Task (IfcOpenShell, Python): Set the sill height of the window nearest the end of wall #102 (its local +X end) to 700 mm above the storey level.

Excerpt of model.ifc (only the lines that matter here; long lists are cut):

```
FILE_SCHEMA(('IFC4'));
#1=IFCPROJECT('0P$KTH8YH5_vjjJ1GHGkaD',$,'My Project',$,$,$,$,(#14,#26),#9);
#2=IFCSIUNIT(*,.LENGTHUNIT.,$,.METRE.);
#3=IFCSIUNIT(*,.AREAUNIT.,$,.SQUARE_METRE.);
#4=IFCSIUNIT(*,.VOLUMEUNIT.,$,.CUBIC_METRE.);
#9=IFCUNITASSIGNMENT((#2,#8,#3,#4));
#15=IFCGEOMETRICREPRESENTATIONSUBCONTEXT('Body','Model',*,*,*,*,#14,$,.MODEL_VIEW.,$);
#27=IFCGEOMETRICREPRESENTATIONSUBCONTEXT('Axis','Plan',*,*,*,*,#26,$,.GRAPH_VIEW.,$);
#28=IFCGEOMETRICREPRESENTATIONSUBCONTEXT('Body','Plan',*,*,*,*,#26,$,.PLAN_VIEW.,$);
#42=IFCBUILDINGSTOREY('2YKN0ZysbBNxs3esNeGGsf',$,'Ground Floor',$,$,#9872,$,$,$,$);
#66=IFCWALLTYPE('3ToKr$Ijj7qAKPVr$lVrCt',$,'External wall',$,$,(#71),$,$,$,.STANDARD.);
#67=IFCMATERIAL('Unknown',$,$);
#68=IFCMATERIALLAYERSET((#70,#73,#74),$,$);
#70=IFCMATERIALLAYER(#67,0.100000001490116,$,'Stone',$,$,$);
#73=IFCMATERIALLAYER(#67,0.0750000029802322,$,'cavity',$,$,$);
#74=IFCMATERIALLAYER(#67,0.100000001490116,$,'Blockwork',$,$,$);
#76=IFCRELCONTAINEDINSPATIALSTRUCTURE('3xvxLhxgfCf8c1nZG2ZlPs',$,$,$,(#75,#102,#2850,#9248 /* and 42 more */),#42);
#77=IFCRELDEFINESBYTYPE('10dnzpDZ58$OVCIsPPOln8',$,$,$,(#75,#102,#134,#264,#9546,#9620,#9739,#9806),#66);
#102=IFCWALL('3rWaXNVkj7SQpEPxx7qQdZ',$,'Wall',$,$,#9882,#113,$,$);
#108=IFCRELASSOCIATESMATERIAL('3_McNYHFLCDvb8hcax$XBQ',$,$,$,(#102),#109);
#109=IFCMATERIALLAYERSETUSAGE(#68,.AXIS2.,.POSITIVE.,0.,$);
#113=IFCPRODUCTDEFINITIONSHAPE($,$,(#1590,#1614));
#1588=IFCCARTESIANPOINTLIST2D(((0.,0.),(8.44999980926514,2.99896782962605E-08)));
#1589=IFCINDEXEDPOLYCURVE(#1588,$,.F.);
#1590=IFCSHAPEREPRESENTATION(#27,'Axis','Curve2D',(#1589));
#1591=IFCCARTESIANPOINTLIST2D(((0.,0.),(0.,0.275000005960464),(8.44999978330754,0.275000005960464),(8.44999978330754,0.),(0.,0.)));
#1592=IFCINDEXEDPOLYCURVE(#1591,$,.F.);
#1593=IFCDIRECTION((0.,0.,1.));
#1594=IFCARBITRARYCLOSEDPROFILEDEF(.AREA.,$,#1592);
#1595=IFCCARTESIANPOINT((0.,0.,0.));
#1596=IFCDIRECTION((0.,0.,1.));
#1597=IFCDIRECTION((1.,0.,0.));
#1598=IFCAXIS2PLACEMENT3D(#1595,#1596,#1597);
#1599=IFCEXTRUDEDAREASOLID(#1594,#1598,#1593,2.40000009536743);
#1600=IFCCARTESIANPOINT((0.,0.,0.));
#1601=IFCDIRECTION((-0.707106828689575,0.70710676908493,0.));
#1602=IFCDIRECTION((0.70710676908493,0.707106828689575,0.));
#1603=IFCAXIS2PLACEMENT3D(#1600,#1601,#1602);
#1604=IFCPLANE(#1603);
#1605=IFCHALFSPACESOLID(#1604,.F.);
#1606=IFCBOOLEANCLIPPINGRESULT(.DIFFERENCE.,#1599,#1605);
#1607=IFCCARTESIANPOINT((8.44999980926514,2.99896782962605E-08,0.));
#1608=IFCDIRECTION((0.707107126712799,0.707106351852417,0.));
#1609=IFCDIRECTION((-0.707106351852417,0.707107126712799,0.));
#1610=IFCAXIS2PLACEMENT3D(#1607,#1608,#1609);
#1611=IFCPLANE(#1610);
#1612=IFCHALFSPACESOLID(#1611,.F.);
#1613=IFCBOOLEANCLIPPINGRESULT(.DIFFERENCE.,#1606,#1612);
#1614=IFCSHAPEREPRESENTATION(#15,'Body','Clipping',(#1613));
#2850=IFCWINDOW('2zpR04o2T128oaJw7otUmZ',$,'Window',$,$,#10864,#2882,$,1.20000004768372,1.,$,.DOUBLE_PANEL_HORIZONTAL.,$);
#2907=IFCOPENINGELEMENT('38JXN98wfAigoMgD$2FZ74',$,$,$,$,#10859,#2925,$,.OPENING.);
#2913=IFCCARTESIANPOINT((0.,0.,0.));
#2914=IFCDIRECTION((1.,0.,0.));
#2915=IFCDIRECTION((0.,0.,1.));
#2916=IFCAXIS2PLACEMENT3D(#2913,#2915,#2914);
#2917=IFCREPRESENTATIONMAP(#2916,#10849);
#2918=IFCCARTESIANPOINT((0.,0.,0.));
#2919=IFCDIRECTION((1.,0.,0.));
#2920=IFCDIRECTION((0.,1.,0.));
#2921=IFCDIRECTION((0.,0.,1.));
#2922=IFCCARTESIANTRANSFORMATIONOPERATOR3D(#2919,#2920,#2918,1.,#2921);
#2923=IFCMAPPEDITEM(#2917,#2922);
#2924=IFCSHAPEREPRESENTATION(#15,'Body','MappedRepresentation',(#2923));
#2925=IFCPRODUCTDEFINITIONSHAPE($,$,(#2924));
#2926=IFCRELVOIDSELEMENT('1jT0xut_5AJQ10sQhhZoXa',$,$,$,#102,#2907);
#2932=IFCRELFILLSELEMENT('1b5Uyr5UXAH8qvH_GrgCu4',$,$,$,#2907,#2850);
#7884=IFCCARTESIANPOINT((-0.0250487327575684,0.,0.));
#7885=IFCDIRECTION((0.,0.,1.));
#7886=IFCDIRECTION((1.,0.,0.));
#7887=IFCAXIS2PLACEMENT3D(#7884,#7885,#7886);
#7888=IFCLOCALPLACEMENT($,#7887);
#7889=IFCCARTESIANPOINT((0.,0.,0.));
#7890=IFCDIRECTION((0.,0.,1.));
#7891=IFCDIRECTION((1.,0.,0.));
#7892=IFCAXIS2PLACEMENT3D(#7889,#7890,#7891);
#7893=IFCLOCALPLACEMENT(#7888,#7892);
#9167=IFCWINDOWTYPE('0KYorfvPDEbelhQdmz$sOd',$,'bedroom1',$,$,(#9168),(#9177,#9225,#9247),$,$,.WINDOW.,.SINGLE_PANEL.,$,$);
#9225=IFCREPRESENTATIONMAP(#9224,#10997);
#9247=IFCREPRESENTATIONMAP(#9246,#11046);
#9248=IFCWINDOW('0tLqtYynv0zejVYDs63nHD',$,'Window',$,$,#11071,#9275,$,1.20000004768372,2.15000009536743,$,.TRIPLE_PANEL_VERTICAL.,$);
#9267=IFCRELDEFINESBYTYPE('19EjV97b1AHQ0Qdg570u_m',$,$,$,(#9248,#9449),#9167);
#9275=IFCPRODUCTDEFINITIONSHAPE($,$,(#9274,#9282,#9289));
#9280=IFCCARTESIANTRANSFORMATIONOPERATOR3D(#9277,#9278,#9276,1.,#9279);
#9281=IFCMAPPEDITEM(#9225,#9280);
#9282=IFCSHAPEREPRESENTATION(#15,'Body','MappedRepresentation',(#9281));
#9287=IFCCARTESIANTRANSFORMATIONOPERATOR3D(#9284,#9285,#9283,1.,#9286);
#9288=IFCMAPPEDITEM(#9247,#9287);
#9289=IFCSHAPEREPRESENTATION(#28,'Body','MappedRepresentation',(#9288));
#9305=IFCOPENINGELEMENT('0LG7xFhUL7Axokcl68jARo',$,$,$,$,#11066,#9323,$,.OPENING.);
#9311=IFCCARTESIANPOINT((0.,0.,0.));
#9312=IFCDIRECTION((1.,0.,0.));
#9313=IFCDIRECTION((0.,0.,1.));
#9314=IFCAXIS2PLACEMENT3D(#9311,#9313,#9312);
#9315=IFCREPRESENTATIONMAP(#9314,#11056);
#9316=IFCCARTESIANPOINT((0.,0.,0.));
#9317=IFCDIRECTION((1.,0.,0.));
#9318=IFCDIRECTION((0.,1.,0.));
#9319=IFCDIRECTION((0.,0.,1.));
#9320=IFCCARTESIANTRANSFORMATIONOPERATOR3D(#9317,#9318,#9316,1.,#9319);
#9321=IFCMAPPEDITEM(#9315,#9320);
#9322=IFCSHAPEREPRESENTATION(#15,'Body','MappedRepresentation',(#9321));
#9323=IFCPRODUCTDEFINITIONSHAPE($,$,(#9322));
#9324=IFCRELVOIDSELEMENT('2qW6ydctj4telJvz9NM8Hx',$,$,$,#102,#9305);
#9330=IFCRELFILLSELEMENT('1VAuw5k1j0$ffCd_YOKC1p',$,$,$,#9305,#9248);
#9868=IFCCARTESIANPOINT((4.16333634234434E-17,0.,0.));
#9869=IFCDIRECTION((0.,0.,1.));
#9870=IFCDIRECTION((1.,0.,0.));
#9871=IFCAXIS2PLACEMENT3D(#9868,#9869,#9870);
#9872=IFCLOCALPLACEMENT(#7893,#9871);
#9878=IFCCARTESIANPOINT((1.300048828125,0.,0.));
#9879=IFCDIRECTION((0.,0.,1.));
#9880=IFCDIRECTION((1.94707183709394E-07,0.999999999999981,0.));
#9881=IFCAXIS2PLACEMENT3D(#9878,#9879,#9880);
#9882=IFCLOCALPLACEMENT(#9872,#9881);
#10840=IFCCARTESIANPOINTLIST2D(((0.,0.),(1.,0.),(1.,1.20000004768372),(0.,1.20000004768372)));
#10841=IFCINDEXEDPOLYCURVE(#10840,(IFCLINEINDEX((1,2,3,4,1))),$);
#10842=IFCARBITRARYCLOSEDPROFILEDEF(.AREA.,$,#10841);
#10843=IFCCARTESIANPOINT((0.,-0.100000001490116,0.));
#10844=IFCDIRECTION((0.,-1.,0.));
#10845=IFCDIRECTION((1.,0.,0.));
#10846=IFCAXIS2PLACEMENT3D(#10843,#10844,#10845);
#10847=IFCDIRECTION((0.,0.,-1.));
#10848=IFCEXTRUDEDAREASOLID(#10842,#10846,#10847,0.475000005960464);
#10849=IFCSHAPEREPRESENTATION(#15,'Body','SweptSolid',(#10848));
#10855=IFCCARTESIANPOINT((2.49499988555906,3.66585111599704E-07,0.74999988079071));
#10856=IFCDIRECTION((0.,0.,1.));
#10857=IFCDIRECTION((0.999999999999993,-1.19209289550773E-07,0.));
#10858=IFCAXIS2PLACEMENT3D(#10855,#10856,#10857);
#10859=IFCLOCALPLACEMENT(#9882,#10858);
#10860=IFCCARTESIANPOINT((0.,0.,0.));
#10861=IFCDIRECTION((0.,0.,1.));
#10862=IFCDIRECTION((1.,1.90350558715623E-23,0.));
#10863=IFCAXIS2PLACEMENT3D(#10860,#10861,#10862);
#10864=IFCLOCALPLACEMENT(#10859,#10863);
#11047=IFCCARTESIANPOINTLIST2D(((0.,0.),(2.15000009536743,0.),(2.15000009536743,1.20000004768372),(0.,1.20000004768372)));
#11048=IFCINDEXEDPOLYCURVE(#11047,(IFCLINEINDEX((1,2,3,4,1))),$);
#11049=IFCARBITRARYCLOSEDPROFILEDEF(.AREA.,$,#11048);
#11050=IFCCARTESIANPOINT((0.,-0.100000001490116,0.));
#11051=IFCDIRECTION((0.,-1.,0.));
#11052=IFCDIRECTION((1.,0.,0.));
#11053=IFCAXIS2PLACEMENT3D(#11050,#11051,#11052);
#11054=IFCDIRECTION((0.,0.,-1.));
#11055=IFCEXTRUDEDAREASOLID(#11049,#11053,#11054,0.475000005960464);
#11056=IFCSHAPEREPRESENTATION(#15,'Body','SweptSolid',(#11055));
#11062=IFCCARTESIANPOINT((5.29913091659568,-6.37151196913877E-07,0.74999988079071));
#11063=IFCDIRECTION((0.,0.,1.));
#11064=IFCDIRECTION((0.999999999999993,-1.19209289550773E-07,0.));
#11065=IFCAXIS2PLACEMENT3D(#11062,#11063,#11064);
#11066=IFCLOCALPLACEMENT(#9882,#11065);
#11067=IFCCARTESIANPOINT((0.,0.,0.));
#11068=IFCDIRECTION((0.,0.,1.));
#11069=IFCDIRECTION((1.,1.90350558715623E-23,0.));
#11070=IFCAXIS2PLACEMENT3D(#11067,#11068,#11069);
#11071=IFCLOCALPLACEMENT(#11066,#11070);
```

```python
import numpy as np
import ifcopenshell
import ifcopenshell.api.geometry
import ifcopenshell.geom
import ifcopenshell.util.element
import ifcopenshell.util.placement
import ifcopenshell.util.shape
import ifcopenshell.util.unit

model = ifcopenshell.open("model.ifc")
unit_scale = ifcopenshell.util.unit.calculate_unit_scale(model)

window = model.by_guid("0tLqtYynv0zejVYDs63nHD")
opening = window.FillsVoids[0].RelatingOpeningElement
storey = ifcopenshell.util.element.get_container(window, ifc_class="IfcBuildingStorey")
level = ifcopenshell.util.placement.get_local_placement(storey.ObjectPlacement)[2, 3]

# The opening's origin need not be at the sill, so measure its lowest point.
shape = ifcopenshell.geom.create_shape(ifcopenshell.geom.settings(), opening)
bottom = ifcopenshell.util.shape.get_shape_bottom_elevation(shape, shape.geometry) / unit_scale
dz = level + 0.7 / unit_scale - bottom

shift = np.array([0.0, 0.0, dz])
# The window is placed relative to its opening, so it follows when the opening moves.
matrix = ifcopenshell.util.placement.get_local_placement(opening.ObjectPlacement)
matrix[:3, 3] += shift
ifcopenshell.api.geometry.edit_object_placement(
    model, product=opening, matrix=matrix, is_si=False, should_transform_children=True
)

print(f"moved by {dz * unit_scale:+.3f} m")

model.write("model_v2.ifc")
```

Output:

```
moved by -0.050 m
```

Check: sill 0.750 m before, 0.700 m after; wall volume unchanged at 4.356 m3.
